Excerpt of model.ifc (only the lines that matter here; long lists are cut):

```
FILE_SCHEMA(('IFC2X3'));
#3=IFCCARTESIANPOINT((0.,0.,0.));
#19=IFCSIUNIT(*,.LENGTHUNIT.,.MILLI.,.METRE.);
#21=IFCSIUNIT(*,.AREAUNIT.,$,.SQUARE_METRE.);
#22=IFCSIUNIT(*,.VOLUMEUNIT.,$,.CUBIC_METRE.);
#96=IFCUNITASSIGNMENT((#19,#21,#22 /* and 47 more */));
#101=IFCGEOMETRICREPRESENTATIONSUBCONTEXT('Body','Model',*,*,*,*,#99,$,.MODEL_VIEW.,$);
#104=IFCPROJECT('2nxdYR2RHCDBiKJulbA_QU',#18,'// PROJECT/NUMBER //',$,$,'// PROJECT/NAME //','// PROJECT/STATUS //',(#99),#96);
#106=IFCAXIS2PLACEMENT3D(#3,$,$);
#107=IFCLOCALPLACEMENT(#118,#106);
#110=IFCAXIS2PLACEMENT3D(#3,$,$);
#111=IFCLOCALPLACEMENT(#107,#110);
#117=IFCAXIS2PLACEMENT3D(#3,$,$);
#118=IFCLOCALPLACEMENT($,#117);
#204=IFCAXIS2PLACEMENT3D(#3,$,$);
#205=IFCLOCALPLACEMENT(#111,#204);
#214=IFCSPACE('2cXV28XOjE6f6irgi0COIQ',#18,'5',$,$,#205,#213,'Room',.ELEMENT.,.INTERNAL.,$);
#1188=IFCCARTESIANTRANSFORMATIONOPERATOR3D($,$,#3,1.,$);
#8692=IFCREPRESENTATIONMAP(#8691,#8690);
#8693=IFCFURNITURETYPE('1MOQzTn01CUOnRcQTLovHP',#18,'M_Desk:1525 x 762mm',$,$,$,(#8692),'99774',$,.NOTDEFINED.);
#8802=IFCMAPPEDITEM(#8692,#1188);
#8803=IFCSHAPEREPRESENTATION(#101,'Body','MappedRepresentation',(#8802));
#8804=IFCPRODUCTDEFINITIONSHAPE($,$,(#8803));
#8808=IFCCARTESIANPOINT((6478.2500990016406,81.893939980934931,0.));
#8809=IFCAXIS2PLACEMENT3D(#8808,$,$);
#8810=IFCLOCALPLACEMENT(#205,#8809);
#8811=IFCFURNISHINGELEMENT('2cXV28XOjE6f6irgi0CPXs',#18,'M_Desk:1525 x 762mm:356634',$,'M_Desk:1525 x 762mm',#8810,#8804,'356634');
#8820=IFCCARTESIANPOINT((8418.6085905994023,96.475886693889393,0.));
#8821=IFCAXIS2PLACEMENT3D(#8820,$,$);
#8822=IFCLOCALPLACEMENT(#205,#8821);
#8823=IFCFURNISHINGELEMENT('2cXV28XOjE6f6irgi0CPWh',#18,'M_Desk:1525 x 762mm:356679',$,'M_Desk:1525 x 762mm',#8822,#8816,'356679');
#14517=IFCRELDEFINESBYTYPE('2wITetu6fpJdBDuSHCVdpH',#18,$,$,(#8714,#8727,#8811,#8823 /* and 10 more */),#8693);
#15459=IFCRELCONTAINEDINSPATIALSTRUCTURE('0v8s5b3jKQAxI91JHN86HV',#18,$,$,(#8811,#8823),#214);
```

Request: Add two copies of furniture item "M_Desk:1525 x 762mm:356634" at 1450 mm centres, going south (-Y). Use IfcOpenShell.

```python
import numpy as np
import ifcopenshell
import ifcopenshell.api.geometry
import ifcopenshell.api.root
import ifcopenshell.util.element
import ifcopenshell.util.placement
import ifcopenshell.util.unit

model = ifcopenshell.open("model.ifc")
unit_scale = ifcopenshell.util.unit.calculate_unit_scale(model)


def reuse_history(source, copy):
    """copy_class also copies each property set's owner history, people and application; keep the originals."""
    for rel in copy.IsDefinedBy:
        if rel.is_a("IfcRelDefinesByProperties") and (history := rel.RelatingPropertyDefinition.OwnerHistory):
            rel.RelatingPropertyDefinition.OwnerHistory = source.OwnerHistory
            ifcopenshell.util.element.remove_deep2(model, history)


source = model.by_guid("2cXV28XOjE6f6irgi0CPXs")
base = ifcopenshell.util.placement.get_local_placement(source.ObjectPlacement)
step = np.array([0.0, -1.0, 0.0]) * 1.45 / unit_scale

for i in range(1, 3):
    copy = ifcopenshell.api.root.copy_class(model, product=source)
    copy.Representation = ifcopenshell.util.element.copy_deep(
        model, source.Representation, exclude=["IfcGeometricRepresentationContext", "IfcRepresentationMap"]
    )
    copy.Name = "M_Desk:1525 x 762mm"
    copy.Tag = None
    reuse_history(source, copy)
    matrix = base.copy()
    matrix[:3, 3] += i * step
    print("added at", matrix[:3, 3].round(3) + 0.0)
    ifcopenshell.api.geometry.edit_object_placement(model, product=copy, matrix=matrix, is_si=False)

model.write("model-out.ifc")
```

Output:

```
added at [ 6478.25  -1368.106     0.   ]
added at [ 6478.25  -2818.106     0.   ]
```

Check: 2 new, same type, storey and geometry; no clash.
